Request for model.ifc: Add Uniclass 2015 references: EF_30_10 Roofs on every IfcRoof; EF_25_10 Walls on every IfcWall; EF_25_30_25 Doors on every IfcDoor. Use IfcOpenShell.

First a look at what the model holds.

```python
import ifcopenshell

model = ifcopenshell.open("model.ifc")
print(model.schema)
print("classifications:", [c.Name for c in model.by_type("IfcClassification")])
for ifc_class in ("IfcDoor", "IfcRoof", "IfcStair", "IfcWall", "IfcWindow"):
    print(ifc_class, len(model.by_type(ifc_class)))
```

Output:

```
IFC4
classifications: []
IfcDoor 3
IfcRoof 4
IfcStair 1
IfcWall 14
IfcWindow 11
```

```python
import ifcopenshell
import ifcopenshell.api.classification

model = ifcopenshell.open("model.ifc")

system = ifcopenshell.api.classification.add_classification(model, classification="Uniclass 2015")

codes = {
    "IfcRoof": ("EF_30_10", "Roofs"),
    "IfcWall": ("EF_25_10", "Walls"),
    "IfcDoor": ("EF_25_30_25", "Doors"),
}
for ifc_class, (code, name) in codes.items():
    products = model.by_type(ifc_class)
    ifcopenshell.api.classification.add_reference(
        model, products=products, classification=system, identification=code, name=name
    )
    print(code, len(products))

model.write("model_edited.ifc")
```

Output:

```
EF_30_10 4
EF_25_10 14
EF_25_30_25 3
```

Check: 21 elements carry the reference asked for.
